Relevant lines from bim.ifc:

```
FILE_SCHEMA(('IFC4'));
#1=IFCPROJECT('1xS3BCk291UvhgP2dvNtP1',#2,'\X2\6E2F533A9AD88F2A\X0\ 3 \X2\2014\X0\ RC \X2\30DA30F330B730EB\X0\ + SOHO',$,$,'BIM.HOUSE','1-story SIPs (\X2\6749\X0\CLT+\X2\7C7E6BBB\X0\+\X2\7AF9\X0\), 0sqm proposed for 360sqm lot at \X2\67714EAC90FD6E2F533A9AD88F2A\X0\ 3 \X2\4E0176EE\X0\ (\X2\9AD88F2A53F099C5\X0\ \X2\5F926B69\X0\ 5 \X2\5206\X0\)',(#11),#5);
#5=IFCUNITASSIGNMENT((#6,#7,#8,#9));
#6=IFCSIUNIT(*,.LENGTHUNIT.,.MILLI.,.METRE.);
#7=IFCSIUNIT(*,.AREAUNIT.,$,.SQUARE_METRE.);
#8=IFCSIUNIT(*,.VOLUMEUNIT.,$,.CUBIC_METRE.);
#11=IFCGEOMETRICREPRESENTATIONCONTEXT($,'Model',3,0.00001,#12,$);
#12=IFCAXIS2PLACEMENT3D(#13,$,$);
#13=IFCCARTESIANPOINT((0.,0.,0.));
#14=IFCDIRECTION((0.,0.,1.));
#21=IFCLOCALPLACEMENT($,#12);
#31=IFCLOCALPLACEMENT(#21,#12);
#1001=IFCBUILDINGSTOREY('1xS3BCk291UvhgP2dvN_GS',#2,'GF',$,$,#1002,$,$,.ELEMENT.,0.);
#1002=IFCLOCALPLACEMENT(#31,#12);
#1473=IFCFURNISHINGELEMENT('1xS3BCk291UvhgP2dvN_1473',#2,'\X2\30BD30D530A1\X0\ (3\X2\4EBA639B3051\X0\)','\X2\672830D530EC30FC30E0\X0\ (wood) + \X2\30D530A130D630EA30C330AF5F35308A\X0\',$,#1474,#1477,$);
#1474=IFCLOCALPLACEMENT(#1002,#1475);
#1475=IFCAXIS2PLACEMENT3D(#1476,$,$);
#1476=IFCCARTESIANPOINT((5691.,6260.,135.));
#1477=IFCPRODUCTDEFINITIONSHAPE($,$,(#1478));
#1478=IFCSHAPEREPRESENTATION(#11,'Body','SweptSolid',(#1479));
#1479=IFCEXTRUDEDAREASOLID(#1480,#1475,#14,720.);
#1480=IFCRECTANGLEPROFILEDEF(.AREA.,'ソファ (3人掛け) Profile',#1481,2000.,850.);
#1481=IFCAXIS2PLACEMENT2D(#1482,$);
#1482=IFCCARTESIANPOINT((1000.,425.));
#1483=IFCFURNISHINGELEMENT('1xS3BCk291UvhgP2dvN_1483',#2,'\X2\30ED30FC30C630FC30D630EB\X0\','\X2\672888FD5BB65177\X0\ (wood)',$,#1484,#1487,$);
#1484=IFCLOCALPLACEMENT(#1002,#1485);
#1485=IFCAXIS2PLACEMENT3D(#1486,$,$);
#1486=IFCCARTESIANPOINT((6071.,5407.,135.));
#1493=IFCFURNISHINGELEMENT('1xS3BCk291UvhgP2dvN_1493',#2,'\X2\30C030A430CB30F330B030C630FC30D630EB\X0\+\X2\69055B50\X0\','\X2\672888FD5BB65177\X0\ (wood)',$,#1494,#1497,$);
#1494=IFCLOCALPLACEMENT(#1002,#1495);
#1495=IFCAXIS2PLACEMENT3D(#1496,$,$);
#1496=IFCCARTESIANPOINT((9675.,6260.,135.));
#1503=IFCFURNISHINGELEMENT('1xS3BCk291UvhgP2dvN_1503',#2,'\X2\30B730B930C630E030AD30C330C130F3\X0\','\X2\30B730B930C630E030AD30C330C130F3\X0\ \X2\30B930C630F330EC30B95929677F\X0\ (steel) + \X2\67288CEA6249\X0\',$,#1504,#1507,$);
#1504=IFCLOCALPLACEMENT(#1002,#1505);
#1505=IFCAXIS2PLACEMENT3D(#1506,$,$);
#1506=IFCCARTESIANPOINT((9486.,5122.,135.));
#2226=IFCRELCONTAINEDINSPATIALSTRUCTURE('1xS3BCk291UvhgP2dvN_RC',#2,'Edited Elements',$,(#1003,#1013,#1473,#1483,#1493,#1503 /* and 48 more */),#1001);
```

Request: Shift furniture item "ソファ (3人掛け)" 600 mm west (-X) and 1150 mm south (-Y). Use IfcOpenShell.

```python
import ifcopenshell
import ifcopenshell.api.geometry
import ifcopenshell.util.placement
import ifcopenshell.util.unit

model = ifcopenshell.open("bim.ifc")
unit_scale = ifcopenshell.util.unit.calculate_unit_scale(model)

item = model.by_id(1473)
matrix = ifcopenshell.util.placement.get_local_placement(item.ObjectPlacement)
matrix[0, 3] -= 0.6 / unit_scale
matrix[1, 3] -= 1.15 / unit_scale
ifcopenshell.api.geometry.edit_object_placement(model, product=item, matrix=matrix, is_si=False)

print(ifcopenshell.util.placement.get_local_placement(item.ObjectPlacement).round(3) + 0.0)

model.write("bim_rev.ifc")
```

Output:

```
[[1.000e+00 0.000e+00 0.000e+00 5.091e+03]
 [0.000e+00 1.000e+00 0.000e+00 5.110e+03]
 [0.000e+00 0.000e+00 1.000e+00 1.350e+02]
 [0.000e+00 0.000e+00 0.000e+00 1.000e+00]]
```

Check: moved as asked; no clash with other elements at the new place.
